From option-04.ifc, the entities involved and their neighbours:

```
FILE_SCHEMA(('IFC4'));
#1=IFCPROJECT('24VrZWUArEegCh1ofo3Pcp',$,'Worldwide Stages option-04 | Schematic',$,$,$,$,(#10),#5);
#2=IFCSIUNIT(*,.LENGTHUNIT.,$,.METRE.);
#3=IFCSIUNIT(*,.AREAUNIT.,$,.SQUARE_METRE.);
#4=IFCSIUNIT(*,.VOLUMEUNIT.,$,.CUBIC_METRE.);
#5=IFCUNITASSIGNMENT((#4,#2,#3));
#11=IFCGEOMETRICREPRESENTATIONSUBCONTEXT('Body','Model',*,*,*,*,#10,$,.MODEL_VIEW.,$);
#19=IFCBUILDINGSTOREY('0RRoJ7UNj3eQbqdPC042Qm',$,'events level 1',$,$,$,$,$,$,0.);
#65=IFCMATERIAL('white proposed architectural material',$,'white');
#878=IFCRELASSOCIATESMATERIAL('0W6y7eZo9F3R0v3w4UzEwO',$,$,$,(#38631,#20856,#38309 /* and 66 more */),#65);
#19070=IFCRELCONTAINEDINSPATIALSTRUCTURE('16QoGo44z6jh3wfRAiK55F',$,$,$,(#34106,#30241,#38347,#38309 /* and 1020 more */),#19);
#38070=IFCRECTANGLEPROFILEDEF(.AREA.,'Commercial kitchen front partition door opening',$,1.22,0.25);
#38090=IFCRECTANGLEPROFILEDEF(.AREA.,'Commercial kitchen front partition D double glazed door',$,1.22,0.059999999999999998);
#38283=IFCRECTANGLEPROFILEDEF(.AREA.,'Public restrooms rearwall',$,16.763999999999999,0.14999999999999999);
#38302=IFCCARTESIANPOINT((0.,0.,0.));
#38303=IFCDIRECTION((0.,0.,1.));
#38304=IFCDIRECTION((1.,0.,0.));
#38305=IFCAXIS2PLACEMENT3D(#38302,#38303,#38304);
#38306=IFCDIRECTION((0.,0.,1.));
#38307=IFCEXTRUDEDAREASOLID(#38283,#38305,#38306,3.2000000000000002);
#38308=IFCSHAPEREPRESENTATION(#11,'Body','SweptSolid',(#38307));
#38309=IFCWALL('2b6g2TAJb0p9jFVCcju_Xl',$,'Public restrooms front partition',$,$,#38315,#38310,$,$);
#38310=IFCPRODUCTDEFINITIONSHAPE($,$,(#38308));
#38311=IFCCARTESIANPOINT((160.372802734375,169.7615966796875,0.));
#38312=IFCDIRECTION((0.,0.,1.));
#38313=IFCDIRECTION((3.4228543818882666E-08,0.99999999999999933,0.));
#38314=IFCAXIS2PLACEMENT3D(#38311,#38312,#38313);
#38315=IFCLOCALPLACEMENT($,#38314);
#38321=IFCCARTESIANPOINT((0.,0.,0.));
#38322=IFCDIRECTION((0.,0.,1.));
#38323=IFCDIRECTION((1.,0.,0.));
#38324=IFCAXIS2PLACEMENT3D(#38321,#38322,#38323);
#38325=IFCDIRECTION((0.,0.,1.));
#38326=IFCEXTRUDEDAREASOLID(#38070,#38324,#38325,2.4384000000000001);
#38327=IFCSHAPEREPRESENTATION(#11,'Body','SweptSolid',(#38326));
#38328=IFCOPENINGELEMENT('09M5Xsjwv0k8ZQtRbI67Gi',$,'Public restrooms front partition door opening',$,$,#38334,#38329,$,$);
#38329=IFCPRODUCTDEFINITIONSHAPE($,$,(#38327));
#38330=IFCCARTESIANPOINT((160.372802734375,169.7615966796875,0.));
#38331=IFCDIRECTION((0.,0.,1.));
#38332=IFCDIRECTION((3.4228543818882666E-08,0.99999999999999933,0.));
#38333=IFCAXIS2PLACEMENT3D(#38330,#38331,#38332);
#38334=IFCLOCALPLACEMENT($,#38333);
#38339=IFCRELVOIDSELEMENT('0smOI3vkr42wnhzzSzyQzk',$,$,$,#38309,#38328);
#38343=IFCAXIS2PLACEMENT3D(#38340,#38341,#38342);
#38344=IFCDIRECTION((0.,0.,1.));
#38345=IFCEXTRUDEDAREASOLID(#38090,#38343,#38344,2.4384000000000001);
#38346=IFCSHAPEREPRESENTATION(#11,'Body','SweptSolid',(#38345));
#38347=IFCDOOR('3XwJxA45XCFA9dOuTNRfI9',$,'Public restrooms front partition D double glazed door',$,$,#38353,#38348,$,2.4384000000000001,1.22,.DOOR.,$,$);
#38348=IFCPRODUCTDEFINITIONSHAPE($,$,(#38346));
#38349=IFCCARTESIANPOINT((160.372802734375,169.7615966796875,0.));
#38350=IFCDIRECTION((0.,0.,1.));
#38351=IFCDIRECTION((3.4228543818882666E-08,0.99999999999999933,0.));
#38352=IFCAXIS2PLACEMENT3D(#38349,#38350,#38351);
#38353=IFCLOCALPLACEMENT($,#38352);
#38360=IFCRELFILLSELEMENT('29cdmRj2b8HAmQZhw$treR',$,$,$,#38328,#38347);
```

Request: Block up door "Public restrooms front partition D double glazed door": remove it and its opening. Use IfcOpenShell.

```python
import ifcopenshell
import ifcopenshell.api.feature
import ifcopenshell.api.root
import ifcopenshell.geom
import ifcopenshell.util.shape

model = ifcopenshell.open("option-04.ifc")
settings = ifcopenshell.geom.settings()


def volume(element):
    """Net volume in cubic metres, openings subtracted."""
    shape = ifcopenshell.geom.create_shape(settings, element)
    return ifcopenshell.util.shape.get_volume(shape.geometry)


door = model.by_guid("3XwJxA45XCFA9dOuTNRfI9")
opening = door.FillsVoids[0].RelatingOpeningElement
wall = opening.VoidsElements[0].RelatingBuildingElement
before = volume(wall)

ifcopenshell.api.root.remove_product(model, product=door)
ifcopenshell.api.feature.remove_feature(model, feature=opening)

after = volume(wall)

print(f"wall volume {before:.3f} -> {after:.3f} m3")

model.write("option-04_v2.ifc")
```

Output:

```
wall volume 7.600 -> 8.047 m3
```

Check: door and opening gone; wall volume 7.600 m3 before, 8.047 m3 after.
